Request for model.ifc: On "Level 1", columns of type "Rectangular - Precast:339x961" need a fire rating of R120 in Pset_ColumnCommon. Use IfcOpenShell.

First a look at what the model holds.

```python
import ifcopenshell
import ifcopenshell.util.element

model = ifcopenshell.open("model.ifc")
print(model.schema)
storey = next(s for s in model.by_type("IfcBuildingStorey") if s.Name == "Level 1")
columns = [e for e in ifcopenshell.util.element.get_decomposition(storey) if e.is_a("IfcColumn")]
seen = {}
for e in columns:
    element_type = ifcopenshell.util.element.get_type(e)
    key = (element_type.Name if element_type != e and element_type else None, ifcopenshell.util.element.get_pset(e, "Pset_ColumnCommon", "FireRating"))
    seen[key] = seen.get(key, 0) + 1
for (name, value), count in sorted(seen.items(), key=str):
    print(count, "x", name, "|", value)
```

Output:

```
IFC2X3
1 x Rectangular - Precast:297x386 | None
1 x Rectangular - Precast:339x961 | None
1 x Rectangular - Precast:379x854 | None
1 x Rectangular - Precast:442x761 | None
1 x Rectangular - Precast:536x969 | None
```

```python
import ifcopenshell
import ifcopenshell.api.pset
import ifcopenshell.util.element

model = ifcopenshell.open("model.ifc")

storey = next(s for s in model.by_type("IfcBuildingStorey") if s.Name == "Level 1")
columns = [e for e in ifcopenshell.util.element.get_decomposition(storey) if e.is_a("IfcColumn")]

count = 0
for e in columns:
    element_type = ifcopenshell.util.element.get_type(e)
    if element_type in (None, e) or element_type.Name != "Rectangular - Precast:339x961":
        continue
    # add_pset returns the element's existing set when there is one.
    pset = ifcopenshell.api.pset.add_pset(model, product=e, name="Pset_ColumnCommon")
    ifcopenshell.api.pset.edit_pset(model, pset=pset, properties={"FireRating": "R120"})
    count += 1

print(count, "columns updated")

model.write("model_v2.ifc")
```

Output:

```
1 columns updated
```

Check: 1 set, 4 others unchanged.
